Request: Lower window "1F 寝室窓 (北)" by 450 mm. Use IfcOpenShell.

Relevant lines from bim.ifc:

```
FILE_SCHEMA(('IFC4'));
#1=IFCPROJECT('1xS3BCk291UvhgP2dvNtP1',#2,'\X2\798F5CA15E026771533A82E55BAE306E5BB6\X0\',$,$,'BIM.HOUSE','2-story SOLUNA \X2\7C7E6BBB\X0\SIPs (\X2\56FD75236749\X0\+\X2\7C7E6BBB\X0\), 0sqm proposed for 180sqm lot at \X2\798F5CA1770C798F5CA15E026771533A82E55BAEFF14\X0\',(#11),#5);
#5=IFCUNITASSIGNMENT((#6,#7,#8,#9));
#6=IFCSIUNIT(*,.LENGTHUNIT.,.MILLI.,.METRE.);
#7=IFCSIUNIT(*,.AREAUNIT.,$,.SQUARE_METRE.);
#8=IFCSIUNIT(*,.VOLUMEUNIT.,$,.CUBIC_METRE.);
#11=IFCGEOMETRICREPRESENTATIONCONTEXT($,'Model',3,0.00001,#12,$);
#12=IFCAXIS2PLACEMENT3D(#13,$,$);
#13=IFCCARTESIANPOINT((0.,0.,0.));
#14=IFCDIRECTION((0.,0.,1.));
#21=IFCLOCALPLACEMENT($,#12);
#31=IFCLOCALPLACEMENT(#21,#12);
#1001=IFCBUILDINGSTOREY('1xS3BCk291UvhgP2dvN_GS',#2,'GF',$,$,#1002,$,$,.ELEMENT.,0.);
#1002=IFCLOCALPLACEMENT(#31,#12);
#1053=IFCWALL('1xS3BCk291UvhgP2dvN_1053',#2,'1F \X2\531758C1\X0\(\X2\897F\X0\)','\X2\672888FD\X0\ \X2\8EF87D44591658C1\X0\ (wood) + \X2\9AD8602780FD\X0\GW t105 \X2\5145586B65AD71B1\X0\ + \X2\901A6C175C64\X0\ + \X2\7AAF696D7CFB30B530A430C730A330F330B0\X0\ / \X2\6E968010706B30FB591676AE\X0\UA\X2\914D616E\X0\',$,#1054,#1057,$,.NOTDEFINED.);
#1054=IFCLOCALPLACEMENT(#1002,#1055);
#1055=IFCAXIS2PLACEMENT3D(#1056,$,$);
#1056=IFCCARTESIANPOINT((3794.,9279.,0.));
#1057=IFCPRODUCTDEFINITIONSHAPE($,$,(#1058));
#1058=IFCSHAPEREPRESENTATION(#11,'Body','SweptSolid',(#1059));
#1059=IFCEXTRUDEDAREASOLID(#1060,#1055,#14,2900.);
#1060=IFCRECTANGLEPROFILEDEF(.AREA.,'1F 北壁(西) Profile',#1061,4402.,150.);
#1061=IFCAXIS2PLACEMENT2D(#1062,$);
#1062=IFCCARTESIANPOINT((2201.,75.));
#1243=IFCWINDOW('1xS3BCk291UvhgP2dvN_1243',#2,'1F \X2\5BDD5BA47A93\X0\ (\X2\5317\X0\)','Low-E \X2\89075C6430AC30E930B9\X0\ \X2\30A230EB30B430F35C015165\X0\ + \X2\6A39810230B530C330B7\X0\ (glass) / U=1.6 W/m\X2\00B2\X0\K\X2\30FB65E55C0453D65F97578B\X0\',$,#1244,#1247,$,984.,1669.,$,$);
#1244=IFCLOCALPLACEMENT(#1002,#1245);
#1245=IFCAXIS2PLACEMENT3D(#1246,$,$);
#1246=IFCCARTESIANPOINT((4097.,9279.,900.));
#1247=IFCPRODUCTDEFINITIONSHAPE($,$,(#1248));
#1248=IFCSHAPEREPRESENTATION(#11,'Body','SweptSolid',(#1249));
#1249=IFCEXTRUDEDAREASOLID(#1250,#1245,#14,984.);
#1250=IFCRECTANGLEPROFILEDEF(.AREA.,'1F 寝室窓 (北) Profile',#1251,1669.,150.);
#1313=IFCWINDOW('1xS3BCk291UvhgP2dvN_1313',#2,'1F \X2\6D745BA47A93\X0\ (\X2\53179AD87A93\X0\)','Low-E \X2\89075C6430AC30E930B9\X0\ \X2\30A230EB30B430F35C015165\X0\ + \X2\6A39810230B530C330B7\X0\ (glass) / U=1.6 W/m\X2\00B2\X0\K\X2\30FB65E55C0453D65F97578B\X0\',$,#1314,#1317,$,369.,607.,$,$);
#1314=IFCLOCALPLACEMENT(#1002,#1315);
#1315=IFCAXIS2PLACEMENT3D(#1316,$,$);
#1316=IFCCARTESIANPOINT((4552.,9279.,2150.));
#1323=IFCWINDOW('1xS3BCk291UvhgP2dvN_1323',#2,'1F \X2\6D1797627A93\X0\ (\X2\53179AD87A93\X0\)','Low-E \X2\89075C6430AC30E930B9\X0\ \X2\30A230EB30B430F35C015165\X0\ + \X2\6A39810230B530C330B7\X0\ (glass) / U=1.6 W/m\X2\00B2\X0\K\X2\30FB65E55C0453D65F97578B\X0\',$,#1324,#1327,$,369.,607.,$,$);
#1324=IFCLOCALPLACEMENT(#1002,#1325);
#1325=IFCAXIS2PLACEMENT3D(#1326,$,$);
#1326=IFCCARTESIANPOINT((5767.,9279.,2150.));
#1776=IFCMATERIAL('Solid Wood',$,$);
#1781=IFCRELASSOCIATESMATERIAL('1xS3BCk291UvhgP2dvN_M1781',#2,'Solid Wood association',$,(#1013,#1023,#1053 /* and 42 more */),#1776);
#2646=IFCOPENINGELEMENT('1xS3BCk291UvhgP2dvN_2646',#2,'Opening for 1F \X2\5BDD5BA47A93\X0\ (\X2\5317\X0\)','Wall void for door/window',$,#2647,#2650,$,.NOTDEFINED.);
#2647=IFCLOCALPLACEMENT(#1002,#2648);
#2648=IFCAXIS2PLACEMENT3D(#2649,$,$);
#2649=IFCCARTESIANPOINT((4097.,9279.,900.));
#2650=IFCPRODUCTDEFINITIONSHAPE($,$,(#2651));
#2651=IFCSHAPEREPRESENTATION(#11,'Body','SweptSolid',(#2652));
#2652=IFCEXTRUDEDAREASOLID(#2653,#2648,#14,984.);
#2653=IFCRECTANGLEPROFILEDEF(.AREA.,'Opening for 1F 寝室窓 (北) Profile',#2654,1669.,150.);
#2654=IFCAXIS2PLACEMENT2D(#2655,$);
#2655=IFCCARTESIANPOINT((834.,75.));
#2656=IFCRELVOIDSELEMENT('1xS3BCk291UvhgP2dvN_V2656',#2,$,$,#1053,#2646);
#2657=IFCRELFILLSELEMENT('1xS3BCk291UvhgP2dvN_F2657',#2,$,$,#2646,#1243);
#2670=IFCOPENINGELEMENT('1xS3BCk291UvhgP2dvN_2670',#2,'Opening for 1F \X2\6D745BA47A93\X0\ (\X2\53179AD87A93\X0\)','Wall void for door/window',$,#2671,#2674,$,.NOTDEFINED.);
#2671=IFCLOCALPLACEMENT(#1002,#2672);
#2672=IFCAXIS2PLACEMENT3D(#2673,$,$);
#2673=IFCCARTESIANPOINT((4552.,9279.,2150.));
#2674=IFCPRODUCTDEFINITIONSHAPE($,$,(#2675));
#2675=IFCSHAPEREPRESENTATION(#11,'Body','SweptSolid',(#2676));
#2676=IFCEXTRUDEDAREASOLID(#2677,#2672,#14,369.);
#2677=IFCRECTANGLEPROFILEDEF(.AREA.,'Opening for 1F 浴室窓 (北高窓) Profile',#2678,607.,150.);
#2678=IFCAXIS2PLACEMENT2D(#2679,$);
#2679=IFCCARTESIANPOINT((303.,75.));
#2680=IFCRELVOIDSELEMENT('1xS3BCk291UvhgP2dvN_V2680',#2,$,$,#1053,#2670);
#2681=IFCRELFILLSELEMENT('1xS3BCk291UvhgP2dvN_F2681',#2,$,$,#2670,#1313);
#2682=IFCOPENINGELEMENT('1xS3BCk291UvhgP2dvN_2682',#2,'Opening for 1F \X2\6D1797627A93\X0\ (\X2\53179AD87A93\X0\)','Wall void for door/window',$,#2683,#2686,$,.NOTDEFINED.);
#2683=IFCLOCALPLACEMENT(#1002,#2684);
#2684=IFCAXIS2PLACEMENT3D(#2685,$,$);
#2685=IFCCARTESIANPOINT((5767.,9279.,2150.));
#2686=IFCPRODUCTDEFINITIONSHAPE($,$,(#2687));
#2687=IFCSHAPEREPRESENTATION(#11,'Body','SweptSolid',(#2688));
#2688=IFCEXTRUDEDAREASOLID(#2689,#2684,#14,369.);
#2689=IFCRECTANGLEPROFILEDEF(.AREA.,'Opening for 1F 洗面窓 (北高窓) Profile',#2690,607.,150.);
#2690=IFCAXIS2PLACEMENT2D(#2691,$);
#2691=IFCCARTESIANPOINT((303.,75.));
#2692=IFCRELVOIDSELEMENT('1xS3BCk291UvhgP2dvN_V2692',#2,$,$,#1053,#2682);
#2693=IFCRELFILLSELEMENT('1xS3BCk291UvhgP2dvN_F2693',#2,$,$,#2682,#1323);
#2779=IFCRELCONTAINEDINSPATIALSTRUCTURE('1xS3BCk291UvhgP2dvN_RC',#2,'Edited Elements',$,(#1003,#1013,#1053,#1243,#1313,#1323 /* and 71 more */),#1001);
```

```python
import numpy as np
import ifcopenshell
import ifcopenshell.api.geometry
import ifcopenshell.util.placement
import ifcopenshell.util.unit

model = ifcopenshell.open("bim.ifc")
unit_scale = ifcopenshell.util.unit.calculate_unit_scale(model)

window = model.by_id(1243)
opening = window.FillsVoids[0].RelatingOpeningElement
dz = -0.45 / unit_scale

shift = np.array([0.0, 0.0, dz])
# The window is not placed relative to its opening, so move both.
for product in (opening, window):
    matrix = ifcopenshell.util.placement.get_local_placement(product.ObjectPlacement)
    matrix[:3, 3] += shift
    ifcopenshell.api.geometry.edit_object_placement(model, product=product, matrix=matrix, is_si=False)

print(f"moved by {dz * unit_scale:+.3f} m")

model.write("bim_rev.ifc")
```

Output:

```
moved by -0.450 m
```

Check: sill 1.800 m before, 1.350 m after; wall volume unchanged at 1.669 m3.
